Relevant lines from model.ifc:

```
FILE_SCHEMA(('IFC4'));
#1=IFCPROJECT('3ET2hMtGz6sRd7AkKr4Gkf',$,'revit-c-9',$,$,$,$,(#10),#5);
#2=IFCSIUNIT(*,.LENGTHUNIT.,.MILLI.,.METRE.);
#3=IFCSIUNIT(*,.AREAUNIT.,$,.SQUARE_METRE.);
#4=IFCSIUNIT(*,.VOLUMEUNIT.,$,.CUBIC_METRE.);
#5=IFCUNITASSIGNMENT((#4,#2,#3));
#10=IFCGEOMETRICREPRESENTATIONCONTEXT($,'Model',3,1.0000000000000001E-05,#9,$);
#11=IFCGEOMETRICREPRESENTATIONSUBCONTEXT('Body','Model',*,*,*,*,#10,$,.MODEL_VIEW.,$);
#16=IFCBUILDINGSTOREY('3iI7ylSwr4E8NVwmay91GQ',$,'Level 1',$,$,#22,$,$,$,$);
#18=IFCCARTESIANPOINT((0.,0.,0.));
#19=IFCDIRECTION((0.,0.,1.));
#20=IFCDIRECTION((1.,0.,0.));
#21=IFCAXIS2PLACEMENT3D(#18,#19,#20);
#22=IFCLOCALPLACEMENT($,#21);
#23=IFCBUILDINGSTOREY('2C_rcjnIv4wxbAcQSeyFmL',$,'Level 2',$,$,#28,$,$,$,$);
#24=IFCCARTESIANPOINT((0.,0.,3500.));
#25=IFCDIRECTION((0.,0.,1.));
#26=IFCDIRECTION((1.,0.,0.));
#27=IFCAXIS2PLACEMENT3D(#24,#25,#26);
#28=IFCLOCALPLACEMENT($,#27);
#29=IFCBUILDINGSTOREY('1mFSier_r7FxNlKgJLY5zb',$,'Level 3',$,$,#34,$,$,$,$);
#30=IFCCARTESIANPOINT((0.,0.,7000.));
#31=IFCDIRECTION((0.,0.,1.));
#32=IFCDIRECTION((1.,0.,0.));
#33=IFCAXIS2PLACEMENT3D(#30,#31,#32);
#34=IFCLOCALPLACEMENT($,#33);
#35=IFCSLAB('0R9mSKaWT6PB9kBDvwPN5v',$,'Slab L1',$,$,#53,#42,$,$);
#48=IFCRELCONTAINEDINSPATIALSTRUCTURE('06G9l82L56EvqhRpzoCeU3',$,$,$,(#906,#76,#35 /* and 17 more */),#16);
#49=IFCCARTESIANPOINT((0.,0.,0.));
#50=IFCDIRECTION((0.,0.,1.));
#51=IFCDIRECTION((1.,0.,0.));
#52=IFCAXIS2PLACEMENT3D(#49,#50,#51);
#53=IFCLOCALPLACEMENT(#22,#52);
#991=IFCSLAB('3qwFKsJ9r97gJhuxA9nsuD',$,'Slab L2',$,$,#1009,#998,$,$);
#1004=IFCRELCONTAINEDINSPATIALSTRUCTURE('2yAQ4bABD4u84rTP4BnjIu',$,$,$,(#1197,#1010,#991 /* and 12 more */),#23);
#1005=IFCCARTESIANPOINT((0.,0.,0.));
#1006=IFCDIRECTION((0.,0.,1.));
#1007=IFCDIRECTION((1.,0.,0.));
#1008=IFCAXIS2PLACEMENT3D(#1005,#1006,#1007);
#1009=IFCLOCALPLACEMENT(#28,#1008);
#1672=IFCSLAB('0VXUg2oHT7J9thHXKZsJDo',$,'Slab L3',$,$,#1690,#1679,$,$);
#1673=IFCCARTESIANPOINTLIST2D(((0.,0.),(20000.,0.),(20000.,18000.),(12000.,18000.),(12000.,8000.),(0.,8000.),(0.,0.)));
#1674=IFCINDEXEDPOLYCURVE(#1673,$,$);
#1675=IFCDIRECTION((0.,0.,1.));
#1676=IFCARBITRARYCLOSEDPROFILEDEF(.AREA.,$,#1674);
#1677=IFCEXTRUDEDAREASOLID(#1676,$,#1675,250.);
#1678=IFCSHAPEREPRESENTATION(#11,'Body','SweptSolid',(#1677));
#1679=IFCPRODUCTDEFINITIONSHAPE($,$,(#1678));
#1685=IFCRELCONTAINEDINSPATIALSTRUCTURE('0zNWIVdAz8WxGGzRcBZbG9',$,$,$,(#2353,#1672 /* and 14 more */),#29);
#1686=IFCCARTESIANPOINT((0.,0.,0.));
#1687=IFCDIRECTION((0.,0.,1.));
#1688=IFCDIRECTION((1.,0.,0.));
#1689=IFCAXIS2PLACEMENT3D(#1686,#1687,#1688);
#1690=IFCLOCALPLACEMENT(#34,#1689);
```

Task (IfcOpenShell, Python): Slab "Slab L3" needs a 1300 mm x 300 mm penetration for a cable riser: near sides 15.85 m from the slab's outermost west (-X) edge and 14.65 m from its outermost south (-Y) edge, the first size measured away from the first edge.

```python
import numpy as np
import ifcopenshell
import ifcopenshell.api.feature
import ifcopenshell.api.geometry
import ifcopenshell.api.root
import ifcopenshell.geom
import ifcopenshell.util.placement
import ifcopenshell.util.representation
import ifcopenshell.util.shape
import ifcopenshell.util.unit

model = ifcopenshell.open("model.ifc")
unit_scale = ifcopenshell.util.unit.calculate_unit_scale(model)
settings = ifcopenshell.geom.settings()


def volume(element):
    """Net volume in cubic metres, openings subtracted."""
    shape = ifcopenshell.geom.create_shape(settings, element)
    return ifcopenshell.util.shape.get_volume(shape.geometry)


slab = model.by_guid("0VXUg2oHT7J9thHXKZsJDo")
before = volume(slab)

# Extent in the slab's own axes, in metres. The edges named are its -X and -Y sides.
slab_shape = ifcopenshell.geom.create_shape(settings, slab)
vertices = ifcopenshell.util.shape.get_vertices(slab_shape.geometry)
x_min, y_min, bottom = vertices.min(axis=0)
top = vertices[:, 2].max()

opening = ifcopenshell.api.root.create_entity(model, ifc_class="IfcOpeningElement", name="Cable riser opening", predefined_type="OPENING")
context = ifcopenshell.util.representation.get_context(model, "Model", "Body", "MODEL_VIEW")
width, depth = 1.3, 0.3
outline = [(0.0, 0.0), (width, 0.0), (width, depth), (0.0, depth), (0.0, 0.0)]
# Overshoot both faces by 50 mm so the cut is clean.
shape = ifcopenshell.api.geometry.add_slab_representation(
    model, context=context, depth=top - bottom + 0.1, polyline=outline
)
ifcopenshell.api.geometry.assign_representation(model, product=opening, representation=shape)

matrix = ifcopenshell.util.placement.get_local_placement(slab.ObjectPlacement)
matrix[:, 3] = matrix @ np.append(np.array([x_min + 15.85, y_min + 14.65, bottom - 0.05]) / unit_scale, 1.0)
ifcopenshell.api.geometry.edit_object_placement(model, product=opening, matrix=matrix, is_si=False)
ifcopenshell.api.feature.add_feature(model, feature=opening, element=slab)

after = volume(slab)

print(f"slab volume {before:.3f} -> {after:.3f} m3")

model.write("model_rev.ifc")
```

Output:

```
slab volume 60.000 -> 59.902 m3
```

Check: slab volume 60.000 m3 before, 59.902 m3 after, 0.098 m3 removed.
